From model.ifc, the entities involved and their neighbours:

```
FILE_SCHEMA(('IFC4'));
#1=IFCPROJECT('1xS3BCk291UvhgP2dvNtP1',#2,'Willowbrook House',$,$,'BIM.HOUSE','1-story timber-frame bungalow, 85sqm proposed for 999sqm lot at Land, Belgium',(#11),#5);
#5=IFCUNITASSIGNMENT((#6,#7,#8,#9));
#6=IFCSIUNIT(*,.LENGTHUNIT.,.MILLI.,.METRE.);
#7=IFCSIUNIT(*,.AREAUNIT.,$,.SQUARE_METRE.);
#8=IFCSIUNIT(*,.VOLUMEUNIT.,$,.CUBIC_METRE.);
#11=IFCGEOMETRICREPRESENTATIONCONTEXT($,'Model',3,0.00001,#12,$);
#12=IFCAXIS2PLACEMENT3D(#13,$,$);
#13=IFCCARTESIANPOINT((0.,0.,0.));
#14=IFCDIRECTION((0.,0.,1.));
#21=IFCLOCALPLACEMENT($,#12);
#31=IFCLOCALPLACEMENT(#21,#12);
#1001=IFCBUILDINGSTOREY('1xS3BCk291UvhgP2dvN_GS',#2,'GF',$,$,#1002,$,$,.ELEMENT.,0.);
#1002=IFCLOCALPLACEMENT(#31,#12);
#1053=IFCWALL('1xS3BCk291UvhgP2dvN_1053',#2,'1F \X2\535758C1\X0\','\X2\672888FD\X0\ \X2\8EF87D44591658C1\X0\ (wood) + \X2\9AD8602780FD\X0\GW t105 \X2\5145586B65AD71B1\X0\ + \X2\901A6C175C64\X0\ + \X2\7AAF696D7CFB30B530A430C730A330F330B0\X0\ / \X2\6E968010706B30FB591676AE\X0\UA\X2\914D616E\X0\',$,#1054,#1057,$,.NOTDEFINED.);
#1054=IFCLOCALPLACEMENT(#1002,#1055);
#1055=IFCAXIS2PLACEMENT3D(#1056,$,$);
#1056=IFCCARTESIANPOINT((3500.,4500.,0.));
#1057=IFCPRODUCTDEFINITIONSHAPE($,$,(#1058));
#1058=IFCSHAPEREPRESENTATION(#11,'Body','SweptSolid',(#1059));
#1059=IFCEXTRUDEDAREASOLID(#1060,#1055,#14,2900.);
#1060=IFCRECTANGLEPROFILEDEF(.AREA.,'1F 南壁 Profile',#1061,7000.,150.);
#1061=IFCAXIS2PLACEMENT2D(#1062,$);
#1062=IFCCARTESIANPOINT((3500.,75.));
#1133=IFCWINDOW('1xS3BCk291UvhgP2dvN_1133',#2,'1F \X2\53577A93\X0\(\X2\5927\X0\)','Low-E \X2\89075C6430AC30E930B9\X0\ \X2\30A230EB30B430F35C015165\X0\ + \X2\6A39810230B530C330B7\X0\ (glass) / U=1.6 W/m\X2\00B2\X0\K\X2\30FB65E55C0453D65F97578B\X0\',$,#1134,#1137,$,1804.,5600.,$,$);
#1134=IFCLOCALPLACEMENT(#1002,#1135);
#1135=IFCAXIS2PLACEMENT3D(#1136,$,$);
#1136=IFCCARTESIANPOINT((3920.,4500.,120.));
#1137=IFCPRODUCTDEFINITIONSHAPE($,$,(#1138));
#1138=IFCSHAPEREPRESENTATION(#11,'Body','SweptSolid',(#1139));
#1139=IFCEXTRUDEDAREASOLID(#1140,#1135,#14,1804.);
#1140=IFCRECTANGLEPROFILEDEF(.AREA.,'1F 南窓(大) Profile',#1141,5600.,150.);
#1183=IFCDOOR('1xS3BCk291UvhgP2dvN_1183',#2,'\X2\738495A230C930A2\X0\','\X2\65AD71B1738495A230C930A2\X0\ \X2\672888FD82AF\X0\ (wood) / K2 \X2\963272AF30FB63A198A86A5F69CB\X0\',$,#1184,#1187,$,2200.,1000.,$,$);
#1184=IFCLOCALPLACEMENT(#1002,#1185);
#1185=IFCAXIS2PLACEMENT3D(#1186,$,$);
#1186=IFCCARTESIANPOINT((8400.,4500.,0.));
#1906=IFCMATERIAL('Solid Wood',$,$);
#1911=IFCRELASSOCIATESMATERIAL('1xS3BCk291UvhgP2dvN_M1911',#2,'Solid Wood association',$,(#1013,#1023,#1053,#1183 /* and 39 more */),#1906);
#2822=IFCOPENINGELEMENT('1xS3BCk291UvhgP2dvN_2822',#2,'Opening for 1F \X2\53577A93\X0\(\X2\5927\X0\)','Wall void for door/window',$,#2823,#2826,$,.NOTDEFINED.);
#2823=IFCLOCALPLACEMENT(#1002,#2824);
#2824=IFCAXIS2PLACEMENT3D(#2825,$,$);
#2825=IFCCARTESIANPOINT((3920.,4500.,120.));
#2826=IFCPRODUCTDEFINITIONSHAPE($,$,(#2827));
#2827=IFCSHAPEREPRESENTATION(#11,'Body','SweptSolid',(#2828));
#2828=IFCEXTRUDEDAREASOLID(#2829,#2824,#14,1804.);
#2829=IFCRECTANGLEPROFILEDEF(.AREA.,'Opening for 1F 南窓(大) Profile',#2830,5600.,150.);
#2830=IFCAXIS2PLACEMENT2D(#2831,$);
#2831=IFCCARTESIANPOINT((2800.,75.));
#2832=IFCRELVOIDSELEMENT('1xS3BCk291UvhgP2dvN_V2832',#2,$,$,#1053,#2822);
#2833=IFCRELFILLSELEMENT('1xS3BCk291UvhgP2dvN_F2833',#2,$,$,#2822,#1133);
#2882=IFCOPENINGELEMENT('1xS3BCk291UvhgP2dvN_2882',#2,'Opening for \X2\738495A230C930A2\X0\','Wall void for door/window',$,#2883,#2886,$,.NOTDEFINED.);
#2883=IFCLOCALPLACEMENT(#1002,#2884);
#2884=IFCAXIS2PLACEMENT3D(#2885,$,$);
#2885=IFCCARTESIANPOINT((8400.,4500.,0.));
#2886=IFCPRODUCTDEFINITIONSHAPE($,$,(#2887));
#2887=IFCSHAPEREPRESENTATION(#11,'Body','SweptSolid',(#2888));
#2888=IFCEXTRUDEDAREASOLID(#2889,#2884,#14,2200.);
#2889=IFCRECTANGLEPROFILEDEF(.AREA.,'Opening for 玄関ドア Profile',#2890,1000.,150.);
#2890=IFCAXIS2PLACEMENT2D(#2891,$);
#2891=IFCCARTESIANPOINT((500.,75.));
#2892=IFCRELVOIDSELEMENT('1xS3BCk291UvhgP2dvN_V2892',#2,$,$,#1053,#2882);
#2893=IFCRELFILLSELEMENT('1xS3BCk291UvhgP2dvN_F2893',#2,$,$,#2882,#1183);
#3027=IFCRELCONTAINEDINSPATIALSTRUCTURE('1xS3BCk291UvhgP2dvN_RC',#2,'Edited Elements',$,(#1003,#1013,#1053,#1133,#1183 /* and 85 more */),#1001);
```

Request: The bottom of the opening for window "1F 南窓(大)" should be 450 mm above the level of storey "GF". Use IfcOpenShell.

```python
import numpy as np
import ifcopenshell
import ifcopenshell.api.geometry
import ifcopenshell.geom
import ifcopenshell.util.element
import ifcopenshell.util.placement
import ifcopenshell.util.shape
import ifcopenshell.util.unit

model = ifcopenshell.open("model.ifc")
unit_scale = ifcopenshell.util.unit.calculate_unit_scale(model)

window = model.by_id(1133)
opening = window.FillsVoids[0].RelatingOpeningElement
storey = ifcopenshell.util.element.get_container(window, ifc_class="IfcBuildingStorey")
level = ifcopenshell.util.placement.get_local_placement(storey.ObjectPlacement)[2, 3]

# The opening's origin need not be at the sill, so measure its lowest point.
shape = ifcopenshell.geom.create_shape(ifcopenshell.geom.settings(), opening)
bottom = ifcopenshell.util.shape.get_shape_bottom_elevation(shape, shape.geometry) / unit_scale
dz = level + 0.45 / unit_scale - bottom

shift = np.array([0.0, 0.0, dz])
# The window is not placed relative to its opening, so move both.
for product in (opening, window):
    matrix = ifcopenshell.util.placement.get_local_placement(product.ObjectPlacement)
    matrix[:3, 3] += shift
    ifcopenshell.api.geometry.edit_object_placement(model, product=product, matrix=matrix, is_si=False)

print(f"moved by {dz * unit_scale:+.3f} m")

model.write("model_updated.ifc")
```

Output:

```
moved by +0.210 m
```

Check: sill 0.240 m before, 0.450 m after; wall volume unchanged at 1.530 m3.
